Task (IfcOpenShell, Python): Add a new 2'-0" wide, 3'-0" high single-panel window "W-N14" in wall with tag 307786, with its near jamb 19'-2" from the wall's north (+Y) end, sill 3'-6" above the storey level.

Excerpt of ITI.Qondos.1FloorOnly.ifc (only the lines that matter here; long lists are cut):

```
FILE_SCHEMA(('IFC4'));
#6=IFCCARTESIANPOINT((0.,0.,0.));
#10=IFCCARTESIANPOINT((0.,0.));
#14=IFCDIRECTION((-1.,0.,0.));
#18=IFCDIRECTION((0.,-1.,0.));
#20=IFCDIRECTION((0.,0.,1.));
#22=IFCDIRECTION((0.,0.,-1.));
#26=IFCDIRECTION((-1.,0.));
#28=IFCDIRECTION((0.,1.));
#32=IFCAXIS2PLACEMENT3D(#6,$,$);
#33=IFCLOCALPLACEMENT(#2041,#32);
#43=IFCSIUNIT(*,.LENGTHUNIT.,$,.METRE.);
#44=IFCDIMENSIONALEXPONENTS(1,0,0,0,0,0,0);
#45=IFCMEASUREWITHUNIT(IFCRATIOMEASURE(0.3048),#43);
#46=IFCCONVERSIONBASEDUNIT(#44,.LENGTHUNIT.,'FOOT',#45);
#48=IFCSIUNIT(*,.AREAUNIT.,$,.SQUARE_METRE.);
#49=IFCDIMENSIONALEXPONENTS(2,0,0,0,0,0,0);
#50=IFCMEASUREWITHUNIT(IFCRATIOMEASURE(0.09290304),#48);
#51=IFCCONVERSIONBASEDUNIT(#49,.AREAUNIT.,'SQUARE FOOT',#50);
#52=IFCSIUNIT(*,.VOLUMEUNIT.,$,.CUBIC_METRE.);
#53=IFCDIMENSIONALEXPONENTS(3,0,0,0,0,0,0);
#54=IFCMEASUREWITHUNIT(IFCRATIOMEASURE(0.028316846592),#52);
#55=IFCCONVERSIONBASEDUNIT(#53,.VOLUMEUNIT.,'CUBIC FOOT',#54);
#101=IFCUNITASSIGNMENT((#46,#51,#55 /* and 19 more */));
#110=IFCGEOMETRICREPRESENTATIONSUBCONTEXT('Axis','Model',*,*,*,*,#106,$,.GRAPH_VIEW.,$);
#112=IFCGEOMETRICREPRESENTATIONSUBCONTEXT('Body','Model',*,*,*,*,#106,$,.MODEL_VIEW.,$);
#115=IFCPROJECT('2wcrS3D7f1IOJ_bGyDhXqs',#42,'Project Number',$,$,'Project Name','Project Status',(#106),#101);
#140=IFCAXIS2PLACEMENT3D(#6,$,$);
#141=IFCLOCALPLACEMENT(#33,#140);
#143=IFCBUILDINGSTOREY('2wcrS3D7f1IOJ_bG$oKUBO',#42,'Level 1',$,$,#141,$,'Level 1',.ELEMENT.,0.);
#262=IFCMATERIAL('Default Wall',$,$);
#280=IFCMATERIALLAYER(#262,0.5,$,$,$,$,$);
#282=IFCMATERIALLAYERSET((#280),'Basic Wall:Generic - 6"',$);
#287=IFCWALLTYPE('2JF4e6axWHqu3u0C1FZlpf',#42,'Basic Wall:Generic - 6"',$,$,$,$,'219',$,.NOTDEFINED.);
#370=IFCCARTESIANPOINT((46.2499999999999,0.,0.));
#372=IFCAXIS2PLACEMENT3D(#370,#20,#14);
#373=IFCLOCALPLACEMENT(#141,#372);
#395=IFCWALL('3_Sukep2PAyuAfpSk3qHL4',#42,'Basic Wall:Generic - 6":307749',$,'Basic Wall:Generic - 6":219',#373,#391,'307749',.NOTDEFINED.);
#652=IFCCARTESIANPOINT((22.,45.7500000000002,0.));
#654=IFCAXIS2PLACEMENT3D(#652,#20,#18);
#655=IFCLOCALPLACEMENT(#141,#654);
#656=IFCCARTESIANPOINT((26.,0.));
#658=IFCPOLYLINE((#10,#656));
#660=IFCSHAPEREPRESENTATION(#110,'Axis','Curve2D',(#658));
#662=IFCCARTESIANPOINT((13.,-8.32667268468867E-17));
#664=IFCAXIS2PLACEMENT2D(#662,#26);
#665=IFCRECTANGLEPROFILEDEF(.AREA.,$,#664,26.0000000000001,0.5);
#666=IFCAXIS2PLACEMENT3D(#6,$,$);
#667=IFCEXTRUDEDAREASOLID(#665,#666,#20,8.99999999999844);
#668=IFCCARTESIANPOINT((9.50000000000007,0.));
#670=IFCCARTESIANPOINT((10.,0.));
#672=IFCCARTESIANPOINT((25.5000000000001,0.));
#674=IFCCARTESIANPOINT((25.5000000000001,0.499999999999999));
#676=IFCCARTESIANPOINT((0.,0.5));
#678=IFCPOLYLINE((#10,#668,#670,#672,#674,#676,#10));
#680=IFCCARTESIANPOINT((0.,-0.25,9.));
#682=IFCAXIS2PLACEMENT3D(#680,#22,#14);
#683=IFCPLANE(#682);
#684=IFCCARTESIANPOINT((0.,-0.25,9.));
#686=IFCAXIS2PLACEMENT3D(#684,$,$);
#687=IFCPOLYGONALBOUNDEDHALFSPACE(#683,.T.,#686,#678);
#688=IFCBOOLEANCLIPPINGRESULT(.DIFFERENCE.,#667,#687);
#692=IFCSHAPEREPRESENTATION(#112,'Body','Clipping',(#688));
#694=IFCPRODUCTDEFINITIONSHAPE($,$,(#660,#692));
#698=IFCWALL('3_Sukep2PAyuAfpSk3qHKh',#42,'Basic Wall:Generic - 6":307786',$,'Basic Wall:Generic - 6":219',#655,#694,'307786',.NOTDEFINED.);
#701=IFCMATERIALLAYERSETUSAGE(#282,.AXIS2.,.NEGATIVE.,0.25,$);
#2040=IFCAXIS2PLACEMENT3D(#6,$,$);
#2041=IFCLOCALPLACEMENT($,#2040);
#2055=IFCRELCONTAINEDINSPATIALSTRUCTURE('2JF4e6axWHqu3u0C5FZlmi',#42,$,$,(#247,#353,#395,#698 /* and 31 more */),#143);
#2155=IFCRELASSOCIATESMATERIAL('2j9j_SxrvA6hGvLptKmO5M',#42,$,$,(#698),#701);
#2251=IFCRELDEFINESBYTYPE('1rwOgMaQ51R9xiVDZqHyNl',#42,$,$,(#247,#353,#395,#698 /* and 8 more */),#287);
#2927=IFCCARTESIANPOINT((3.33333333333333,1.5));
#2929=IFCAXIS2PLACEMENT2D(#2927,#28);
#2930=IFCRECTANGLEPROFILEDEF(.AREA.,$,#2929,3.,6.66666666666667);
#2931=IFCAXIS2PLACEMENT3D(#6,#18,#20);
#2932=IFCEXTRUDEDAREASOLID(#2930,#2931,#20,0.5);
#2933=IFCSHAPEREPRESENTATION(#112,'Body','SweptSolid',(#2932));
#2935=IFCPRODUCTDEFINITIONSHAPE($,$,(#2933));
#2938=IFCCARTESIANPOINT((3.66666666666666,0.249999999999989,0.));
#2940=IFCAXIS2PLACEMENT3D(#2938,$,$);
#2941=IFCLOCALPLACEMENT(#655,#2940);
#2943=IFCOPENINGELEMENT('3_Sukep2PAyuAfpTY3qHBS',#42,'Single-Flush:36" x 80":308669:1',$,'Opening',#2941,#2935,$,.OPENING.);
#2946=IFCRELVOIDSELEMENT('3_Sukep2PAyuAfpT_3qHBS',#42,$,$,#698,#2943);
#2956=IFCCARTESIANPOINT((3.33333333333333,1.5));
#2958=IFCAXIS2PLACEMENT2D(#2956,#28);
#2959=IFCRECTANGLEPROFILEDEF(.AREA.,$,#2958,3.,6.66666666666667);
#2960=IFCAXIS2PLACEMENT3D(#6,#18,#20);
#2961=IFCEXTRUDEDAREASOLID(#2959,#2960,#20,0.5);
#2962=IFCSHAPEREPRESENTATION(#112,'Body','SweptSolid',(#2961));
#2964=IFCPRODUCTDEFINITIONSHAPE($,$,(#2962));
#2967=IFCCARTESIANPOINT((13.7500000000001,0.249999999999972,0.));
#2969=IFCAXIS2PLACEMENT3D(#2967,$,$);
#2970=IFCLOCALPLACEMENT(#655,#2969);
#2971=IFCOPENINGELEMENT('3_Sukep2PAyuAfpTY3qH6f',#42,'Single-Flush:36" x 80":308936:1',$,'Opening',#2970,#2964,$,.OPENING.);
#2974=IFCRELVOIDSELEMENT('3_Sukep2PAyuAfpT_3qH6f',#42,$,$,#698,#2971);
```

```python
import numpy as np
import ifcopenshell
import ifcopenshell.api.feature
import ifcopenshell.api.geometry
import ifcopenshell.api.root
import ifcopenshell.api.spatial
import ifcopenshell.geom
import ifcopenshell.util.element
import ifcopenshell.util.placement
import ifcopenshell.util.representation
import ifcopenshell.util.shape
import ifcopenshell.util.unit

model = ifcopenshell.open("ITI.Qondos.1FloorOnly.ifc")
unit_scale = ifcopenshell.util.unit.calculate_unit_scale(model)
settings = ifcopenshell.geom.settings()


def volume(element):
    """Net volume in cubic metres, openings subtracted."""
    shape = ifcopenshell.geom.create_shape(settings, element)
    return ifcopenshell.util.shape.get_volume(shape.geometry)


wall = model.by_guid("3_Sukep2PAyuAfpSk3qHKh")
storey = ifcopenshell.util.element.get_container(wall, ifc_class="IfcBuildingStorey")
context = ifcopenshell.util.representation.get_context(model, "Model", "Body", "MODEL_VIEW")
before = volume(wall)

width, height, from_end, sill = 0.6096, 0.9144, 5.842, 1.0668  # metres

# The wall runs along its own X axis, and the end named is its -X end.
wall_shape = ifcopenshell.geom.create_shape(settings, wall)
x, y, z = ifcopenshell.util.shape.get_vertices(wall_shape.geometry).T
start = x.min() + from_end
face, thickness = float(y.min()), float(y.max() - y.min())
wall_matrix = ifcopenshell.util.placement.get_local_placement(wall.ObjectPlacement)
level = ifcopenshell.util.placement.get_local_placement(storey.ObjectPlacement)[2, 3]


def in_wall(x, y):
    """Placement at x, y metres in the wall's axes, at sill height."""
    matrix = wall_matrix.copy()
    matrix[:, 3] = wall_matrix @ np.array([x / unit_scale, y / unit_scale, 0.0, 1.0])
    matrix[2, 3] = level + sill / unit_scale
    return matrix


# Opening: a box that overshoots both wall faces by 50 mm.
opening = ifcopenshell.api.root.create_entity(model, ifc_class="IfcOpeningElement", predefined_type="OPENING")
box = ifcopenshell.api.geometry.add_wall_representation(
    model, context=context, length=width, height=height, thickness=thickness + 0.1
)
ifcopenshell.api.geometry.assign_representation(model, product=opening, representation=box)
ifcopenshell.api.geometry.edit_object_placement(model, product=opening, matrix=in_wall(start, face - 0.05), is_si=False)
ifcopenshell.api.feature.add_feature(model, feature=opening, element=wall)

window = ifcopenshell.api.root.create_entity(model, ifc_class="IfcWindow", name="W-N14", predefined_type="WINDOW")
window.OverallWidth, window.OverallHeight = width / unit_scale, height / unit_scale
window.PartitioningType = "SINGLE_PANEL"
body = ifcopenshell.api.geometry.add_window_representation(
    model,
    context=context,
    overall_width=window.OverallWidth,
    overall_height=window.OverallHeight,
    partition_type="SINGLE_PANEL",
)
ifcopenshell.api.geometry.assign_representation(model, product=window, representation=body)
ifcopenshell.api.spatial.assign_container(model, products=[window], relating_structure=storey)
ifcopenshell.api.feature.add_filling(model, opening=opening, element=window)

# Centre the window in the wall's thickness.
ifcopenshell.api.geometry.edit_object_placement(model, product=window, matrix=in_wall(start, face), is_si=False)
window_shape = ifcopenshell.geom.create_shape(settings, window)
depth = ifcopenshell.util.shape.get_vertices(window_shape.geometry)[:, 1]
offset = face + thickness / 2 - (depth.min() + depth.max()) / 2
ifcopenshell.api.geometry.edit_object_placement(model, product=window, matrix=in_wall(start, offset), is_si=False)

after = volume(wall)

print(f"wall volume {before:.3f} -> {after:.3f} m3")

model.write("ITI.Qondos.1FloorOnly_v2.ifc")
```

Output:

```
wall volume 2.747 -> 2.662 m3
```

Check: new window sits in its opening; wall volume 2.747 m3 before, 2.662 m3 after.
